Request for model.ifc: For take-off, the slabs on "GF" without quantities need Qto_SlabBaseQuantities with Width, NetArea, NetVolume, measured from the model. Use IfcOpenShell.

First a look at what the model holds.

```python
import ifcopenshell
import ifcopenshell.util.element
import ifcopenshell.util.unit

model = ifcopenshell.open("model.ifc")
print(model.schema)
for unit_type in ("LENGTHUNIT", "AREAUNIT", "VOLUMEUNIT"):
    print(unit_type, ifcopenshell.util.unit.calculate_unit_scale(model, unit_type))
storey = next(s for s in model.by_type("IfcBuildingStorey") if s.Name == "GF")
slabs = [e for e in ifcopenshell.util.element.get_decomposition(storey) if e.is_a("IfcSlab")]
for e in sorted(slabs, key=lambda e: e.id()):
    print(e.id(), e.is_a(), e.Name, list(ifcopenshell.util.element.get_psets(e, qtos_only=True)), sep=" | ")
```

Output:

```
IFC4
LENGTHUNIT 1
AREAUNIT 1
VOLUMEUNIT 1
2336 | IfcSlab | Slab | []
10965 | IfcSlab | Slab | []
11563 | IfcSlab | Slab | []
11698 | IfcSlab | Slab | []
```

```python
import ifcopenshell
import ifcopenshell.api.pset
import ifcopenshell.geom
import ifcopenshell.util.element
import ifcopenshell.util.shape
import ifcopenshell.util.unit

model = ifcopenshell.open("model.ifc")
unit_scale = ifcopenshell.util.unit.calculate_unit_scale(model)
area_scale = ifcopenshell.util.unit.calculate_unit_scale(model, "AREAUNIT")
volume_scale = ifcopenshell.util.unit.calculate_unit_scale(model, "VOLUMEUNIT")
settings = ifcopenshell.geom.settings()

storey = next(s for s in model.by_type("IfcBuildingStorey") if s.Name == "GF")
slabs = [e for e in ifcopenshell.util.element.get_decomposition(storey) if e.is_a("IfcSlab")]

for e in sorted(slabs, key=lambda e: e.id()):
    if ifcopenshell.util.element.get_psets(e, qtos_only=True, should_inherit=False):
        continue
    # Geometry comes back in metres, in the element's own axes.
    shape = ifcopenshell.geom.create_shape(settings, e)
    values = {
        "Width": ifcopenshell.util.shape.get_z(shape.geometry) / unit_scale,
        "NetArea": ifcopenshell.util.shape.get_footprint_area(shape.geometry) / area_scale,
        "NetVolume": ifcopenshell.util.shape.get_volume(shape.geometry) / volume_scale,
    }
    qto = ifcopenshell.api.pset.add_qto(model, product=e, name="Qto_SlabBaseQuantities")
    ifcopenshell.api.pset.edit_qto(model, qto=qto, properties=values)
    print(e.id(), {k: round(v, 3) for k, v in values.items()})

model.write("model_rev.ifc")
```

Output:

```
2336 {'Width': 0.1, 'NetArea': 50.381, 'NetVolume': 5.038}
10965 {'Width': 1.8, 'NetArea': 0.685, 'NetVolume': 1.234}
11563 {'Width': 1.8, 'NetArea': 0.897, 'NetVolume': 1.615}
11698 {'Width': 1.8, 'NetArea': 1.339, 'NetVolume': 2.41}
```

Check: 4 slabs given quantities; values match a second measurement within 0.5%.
